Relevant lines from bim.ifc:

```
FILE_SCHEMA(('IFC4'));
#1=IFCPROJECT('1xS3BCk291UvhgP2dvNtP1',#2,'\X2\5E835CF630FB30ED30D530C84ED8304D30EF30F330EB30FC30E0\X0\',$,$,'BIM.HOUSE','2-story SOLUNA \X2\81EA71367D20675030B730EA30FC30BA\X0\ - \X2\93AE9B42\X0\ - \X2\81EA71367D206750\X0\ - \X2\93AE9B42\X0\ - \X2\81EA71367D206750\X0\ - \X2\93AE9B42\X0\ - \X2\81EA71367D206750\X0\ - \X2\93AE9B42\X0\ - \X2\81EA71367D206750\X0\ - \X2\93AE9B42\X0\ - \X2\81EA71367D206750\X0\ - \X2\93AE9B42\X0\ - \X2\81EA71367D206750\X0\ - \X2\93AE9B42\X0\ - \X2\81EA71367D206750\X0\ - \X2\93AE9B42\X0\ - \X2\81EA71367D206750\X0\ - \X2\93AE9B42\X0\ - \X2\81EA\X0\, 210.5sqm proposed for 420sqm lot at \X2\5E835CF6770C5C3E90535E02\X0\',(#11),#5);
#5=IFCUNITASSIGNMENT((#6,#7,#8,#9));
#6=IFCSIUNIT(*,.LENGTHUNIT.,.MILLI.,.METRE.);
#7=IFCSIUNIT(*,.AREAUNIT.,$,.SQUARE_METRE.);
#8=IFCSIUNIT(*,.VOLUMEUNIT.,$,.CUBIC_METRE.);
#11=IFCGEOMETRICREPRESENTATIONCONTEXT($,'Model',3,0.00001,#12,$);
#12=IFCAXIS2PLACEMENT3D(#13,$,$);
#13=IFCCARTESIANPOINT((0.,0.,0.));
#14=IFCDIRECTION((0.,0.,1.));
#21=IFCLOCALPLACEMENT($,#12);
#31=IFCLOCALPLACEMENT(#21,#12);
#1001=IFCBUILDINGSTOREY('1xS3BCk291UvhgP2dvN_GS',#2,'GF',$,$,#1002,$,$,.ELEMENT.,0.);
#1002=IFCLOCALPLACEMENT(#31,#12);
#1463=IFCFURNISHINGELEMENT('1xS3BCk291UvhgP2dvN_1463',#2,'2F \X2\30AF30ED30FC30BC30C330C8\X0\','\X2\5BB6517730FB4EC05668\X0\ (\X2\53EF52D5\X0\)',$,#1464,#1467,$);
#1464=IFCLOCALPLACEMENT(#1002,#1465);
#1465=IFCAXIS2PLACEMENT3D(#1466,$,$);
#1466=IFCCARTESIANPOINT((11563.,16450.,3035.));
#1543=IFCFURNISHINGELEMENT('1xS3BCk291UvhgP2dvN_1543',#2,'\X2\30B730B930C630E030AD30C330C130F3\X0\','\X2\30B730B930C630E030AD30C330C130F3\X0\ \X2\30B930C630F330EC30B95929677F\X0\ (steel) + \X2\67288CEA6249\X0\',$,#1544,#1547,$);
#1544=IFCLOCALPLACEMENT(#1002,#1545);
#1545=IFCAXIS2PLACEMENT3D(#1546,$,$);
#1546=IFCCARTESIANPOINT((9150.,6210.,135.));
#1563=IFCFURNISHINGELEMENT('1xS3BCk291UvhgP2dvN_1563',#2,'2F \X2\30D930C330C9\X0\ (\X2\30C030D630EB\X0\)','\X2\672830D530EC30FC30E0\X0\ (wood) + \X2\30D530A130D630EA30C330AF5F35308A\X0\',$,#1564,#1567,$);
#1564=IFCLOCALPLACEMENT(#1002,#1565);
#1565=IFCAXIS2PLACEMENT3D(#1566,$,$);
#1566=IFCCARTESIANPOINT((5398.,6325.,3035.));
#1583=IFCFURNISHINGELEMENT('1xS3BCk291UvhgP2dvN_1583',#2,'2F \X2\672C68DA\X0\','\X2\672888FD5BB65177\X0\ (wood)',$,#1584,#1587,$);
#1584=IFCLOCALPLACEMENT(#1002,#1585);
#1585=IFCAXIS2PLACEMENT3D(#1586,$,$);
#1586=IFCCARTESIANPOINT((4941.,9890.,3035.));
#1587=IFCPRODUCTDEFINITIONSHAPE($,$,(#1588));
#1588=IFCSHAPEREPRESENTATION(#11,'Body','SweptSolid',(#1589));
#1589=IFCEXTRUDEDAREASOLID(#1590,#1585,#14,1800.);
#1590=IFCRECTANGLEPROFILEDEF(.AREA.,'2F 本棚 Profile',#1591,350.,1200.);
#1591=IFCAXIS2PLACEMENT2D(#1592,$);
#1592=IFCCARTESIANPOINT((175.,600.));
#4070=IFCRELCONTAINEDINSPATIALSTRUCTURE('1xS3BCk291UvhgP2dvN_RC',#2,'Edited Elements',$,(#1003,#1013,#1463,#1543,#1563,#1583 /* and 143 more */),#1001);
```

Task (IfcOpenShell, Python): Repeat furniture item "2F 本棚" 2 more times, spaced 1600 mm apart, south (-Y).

```python
import numpy as np
import ifcopenshell
import ifcopenshell.api.geometry
import ifcopenshell.api.root
import ifcopenshell.util.element
import ifcopenshell.util.placement

model = ifcopenshell.open("bim.ifc")


def reuse_history(source, copy):
    """copy_class also copies each property set's owner history, people and application; keep the originals."""
    for rel in copy.IsDefinedBy:
        if rel.is_a("IfcRelDefinesByProperties") and (history := rel.RelatingPropertyDefinition.OwnerHistory):
            rel.RelatingPropertyDefinition.OwnerHistory = source.OwnerHistory
            ifcopenshell.util.element.remove_deep2(model, history)


source = model.by_id(1583)
base = ifcopenshell.util.placement.get_local_placement(source.ObjectPlacement)
step = np.array([0.0, -1.0, 0.0]) * 1600.0

for i in range(1, 3):
    copy = ifcopenshell.api.root.copy_class(model, product=source)
    copy.Representation = ifcopenshell.util.element.copy_deep(
        model, source.Representation, exclude=["IfcGeometricRepresentationContext", "IfcRepresentationMap"]
    )
    reuse_history(source, copy)
    matrix = base.copy()
    matrix[:3, 3] += i * step
    print("added at", matrix[:3, 3].round(3) + 0.0)
    ifcopenshell.api.geometry.edit_object_placement(model, product=copy, matrix=matrix, is_si=False)

model.write("bim_v2.ifc")
```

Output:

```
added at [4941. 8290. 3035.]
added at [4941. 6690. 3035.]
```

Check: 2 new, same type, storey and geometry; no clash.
